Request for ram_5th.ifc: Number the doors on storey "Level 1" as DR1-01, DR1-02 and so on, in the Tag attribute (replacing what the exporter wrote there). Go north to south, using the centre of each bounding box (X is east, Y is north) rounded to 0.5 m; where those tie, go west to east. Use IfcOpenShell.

First a look at what the model holds.

```python
import ifcopenshell
import ifcopenshell.util.element
import ifcopenshell.util.placement

model = ifcopenshell.open("ram_5th.ifc")
print(model.schema)
storey = next(s for s in model.by_type("IfcBuildingStorey") if s.Name == "Level 1")
doors = [e for e in ifcopenshell.util.element.get_decomposition(storey) if e.is_a("IfcDoor")]
for e in sorted(doors, key=lambda e: e.id()):
    origin = ifcopenshell.util.placement.get_local_placement(e.ObjectPlacement)[:3, 3]
    print(e.id(), e.Tag, e.Name, origin.round(2) + 0.0, sep=" | ")
```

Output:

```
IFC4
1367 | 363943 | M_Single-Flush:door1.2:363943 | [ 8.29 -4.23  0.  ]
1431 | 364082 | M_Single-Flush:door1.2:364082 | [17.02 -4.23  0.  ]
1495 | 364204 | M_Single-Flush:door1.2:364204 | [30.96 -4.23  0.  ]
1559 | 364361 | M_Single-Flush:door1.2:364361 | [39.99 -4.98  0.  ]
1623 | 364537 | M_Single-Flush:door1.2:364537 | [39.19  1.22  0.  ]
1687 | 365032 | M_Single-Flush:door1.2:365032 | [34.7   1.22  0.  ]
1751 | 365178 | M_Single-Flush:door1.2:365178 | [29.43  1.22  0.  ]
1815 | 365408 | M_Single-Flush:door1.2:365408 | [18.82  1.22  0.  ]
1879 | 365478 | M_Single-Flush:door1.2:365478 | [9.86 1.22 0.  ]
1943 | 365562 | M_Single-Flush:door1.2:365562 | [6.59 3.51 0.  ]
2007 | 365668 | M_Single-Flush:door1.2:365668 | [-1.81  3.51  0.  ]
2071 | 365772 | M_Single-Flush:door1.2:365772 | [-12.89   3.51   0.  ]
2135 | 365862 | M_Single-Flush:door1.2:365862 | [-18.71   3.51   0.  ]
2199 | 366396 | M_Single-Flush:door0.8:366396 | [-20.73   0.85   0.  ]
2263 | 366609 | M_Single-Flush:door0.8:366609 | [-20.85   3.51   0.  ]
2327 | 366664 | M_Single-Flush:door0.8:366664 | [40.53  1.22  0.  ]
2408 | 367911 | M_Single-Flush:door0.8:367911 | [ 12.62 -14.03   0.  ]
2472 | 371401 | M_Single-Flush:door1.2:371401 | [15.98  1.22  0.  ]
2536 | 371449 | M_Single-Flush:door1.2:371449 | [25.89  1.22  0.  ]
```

```python
import ifcopenshell
import ifcopenshell.geom
import ifcopenshell.util.element
import ifcopenshell.util.shape

model = ifcopenshell.open("ram_5th.ifc")
settings = ifcopenshell.geom.settings()
settings.set("use-world-coords", True)


def centre(element):
    shape = ifcopenshell.geom.create_shape(settings, element)
    return ifcopenshell.util.shape.get_bbox_centroid(shape.geometry)


storey = next(s for s in model.by_type("IfcBuildingStorey") if s.Name == "Level 1")
doors = [e for e in ifcopenshell.util.element.get_decomposition(storey) if e.is_a("IfcDoor")]

# Insertion points can sit at a corner or the storey origin, so sort by the geometry (in metres).
centres = {e: centre(e) for e in doors}
doors.sort(key=lambda e: (-round(centres[e][1] / 0.5), centres[e][0]))

for i, e in enumerate(doors, start=1):
    number = f"DR1-{i:02d}"
    e.Tag = number
    print(e.id(), number)

model.write("ram_5th-out.ifc")
```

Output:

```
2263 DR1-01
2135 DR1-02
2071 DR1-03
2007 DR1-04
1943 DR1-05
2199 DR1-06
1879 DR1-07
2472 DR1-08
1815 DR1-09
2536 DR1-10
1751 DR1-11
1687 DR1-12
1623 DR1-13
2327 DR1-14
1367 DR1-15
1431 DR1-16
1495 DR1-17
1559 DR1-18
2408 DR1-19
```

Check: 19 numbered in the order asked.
